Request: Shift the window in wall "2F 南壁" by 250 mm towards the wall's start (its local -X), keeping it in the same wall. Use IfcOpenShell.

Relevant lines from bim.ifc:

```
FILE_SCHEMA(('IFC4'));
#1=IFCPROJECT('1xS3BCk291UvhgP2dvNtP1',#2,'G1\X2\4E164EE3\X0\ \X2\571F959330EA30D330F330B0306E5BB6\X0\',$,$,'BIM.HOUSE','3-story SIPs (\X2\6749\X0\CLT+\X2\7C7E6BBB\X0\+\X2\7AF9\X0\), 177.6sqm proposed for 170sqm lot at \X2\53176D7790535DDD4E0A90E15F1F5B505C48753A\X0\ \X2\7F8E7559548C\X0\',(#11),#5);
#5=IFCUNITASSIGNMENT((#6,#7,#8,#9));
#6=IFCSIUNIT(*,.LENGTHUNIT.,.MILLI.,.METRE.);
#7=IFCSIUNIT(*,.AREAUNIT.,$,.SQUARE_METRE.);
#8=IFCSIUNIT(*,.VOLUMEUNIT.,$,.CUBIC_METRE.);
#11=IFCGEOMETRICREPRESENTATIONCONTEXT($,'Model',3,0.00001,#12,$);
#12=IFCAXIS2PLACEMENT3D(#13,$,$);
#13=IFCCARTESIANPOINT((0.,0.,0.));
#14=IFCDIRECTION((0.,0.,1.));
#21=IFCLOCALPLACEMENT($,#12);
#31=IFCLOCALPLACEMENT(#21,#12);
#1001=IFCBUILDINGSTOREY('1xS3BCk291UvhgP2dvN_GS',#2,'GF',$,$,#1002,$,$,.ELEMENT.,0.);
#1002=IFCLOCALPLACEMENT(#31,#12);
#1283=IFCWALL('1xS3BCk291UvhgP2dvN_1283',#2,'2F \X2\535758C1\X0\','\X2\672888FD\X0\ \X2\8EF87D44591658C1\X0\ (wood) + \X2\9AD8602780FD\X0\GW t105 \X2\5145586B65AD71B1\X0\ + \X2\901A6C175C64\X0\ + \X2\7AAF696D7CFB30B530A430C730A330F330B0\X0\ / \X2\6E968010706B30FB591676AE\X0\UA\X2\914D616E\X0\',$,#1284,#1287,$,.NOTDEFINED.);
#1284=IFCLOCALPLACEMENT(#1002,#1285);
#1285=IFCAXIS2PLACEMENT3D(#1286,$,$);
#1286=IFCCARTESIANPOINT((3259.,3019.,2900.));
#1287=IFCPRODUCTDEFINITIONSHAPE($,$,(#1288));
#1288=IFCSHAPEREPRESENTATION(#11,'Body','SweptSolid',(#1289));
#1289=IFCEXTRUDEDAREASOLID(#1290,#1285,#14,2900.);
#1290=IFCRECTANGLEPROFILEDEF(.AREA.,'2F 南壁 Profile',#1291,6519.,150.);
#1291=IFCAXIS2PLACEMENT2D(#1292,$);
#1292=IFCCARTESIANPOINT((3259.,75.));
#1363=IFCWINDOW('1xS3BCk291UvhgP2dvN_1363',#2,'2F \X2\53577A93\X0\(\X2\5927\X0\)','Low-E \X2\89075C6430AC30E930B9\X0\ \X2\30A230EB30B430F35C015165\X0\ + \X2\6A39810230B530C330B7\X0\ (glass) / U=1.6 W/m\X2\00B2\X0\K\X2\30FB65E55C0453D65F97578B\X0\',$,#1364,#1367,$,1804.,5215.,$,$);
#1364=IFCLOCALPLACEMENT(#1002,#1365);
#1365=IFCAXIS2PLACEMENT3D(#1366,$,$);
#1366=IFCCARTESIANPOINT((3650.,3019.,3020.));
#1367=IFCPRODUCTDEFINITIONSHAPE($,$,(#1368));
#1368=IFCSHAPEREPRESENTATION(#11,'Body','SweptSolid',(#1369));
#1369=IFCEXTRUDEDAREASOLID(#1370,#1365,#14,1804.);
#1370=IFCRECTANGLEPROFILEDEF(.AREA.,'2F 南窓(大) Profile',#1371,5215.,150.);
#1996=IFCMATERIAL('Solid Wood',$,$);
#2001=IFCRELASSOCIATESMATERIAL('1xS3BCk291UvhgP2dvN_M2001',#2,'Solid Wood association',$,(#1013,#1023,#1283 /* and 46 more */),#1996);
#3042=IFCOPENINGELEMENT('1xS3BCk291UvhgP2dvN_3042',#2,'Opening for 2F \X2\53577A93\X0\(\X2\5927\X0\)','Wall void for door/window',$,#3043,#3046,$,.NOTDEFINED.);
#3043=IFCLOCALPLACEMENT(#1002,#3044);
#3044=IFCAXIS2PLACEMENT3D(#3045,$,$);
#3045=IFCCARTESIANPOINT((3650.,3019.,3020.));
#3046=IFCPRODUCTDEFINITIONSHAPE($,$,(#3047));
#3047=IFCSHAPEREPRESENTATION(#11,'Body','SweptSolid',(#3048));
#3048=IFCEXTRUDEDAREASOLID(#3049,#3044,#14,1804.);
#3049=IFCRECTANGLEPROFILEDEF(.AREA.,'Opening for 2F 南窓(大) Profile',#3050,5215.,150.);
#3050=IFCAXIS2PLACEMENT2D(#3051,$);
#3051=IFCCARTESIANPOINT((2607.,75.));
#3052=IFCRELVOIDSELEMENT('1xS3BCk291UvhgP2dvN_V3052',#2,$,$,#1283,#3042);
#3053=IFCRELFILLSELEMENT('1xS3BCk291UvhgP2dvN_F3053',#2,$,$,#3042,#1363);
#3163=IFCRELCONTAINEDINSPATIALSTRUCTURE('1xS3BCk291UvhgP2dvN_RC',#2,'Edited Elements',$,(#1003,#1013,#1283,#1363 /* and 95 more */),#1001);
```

```python
import ifcopenshell
import ifcopenshell.api.geometry
import ifcopenshell.util.placement

model = ifcopenshell.open("bim.ifc")

window = model.by_guid("1xS3BCk291UvhgP2dvN_1363")
opening = window.FillsVoids[0].RelatingOpeningElement
wall = opening.VoidsElements[0].RelatingBuildingElement

wall_matrix = ifcopenshell.util.placement.get_local_placement(wall.ObjectPlacement)
shift = wall_matrix[:3, 0] * -250.0
before = ifcopenshell.util.placement.get_local_placement(window.ObjectPlacement)[:3, 3].copy()

# The window is not placed relative to its opening, so move both.
for product in (opening, window):
    matrix = ifcopenshell.util.placement.get_local_placement(product.ObjectPlacement)
    matrix[:3, 3] += shift
    ifcopenshell.api.geometry.edit_object_placement(model, product=product, matrix=matrix, is_si=False)

after = ifcopenshell.util.placement.get_local_placement(window.ObjectPlacement)[:3, 3]
print("window moved by", (after - before).round(3) + 0.0)

model.write("bim-out.ifc")
```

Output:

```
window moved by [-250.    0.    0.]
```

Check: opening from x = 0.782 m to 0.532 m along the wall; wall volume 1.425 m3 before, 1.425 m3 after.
